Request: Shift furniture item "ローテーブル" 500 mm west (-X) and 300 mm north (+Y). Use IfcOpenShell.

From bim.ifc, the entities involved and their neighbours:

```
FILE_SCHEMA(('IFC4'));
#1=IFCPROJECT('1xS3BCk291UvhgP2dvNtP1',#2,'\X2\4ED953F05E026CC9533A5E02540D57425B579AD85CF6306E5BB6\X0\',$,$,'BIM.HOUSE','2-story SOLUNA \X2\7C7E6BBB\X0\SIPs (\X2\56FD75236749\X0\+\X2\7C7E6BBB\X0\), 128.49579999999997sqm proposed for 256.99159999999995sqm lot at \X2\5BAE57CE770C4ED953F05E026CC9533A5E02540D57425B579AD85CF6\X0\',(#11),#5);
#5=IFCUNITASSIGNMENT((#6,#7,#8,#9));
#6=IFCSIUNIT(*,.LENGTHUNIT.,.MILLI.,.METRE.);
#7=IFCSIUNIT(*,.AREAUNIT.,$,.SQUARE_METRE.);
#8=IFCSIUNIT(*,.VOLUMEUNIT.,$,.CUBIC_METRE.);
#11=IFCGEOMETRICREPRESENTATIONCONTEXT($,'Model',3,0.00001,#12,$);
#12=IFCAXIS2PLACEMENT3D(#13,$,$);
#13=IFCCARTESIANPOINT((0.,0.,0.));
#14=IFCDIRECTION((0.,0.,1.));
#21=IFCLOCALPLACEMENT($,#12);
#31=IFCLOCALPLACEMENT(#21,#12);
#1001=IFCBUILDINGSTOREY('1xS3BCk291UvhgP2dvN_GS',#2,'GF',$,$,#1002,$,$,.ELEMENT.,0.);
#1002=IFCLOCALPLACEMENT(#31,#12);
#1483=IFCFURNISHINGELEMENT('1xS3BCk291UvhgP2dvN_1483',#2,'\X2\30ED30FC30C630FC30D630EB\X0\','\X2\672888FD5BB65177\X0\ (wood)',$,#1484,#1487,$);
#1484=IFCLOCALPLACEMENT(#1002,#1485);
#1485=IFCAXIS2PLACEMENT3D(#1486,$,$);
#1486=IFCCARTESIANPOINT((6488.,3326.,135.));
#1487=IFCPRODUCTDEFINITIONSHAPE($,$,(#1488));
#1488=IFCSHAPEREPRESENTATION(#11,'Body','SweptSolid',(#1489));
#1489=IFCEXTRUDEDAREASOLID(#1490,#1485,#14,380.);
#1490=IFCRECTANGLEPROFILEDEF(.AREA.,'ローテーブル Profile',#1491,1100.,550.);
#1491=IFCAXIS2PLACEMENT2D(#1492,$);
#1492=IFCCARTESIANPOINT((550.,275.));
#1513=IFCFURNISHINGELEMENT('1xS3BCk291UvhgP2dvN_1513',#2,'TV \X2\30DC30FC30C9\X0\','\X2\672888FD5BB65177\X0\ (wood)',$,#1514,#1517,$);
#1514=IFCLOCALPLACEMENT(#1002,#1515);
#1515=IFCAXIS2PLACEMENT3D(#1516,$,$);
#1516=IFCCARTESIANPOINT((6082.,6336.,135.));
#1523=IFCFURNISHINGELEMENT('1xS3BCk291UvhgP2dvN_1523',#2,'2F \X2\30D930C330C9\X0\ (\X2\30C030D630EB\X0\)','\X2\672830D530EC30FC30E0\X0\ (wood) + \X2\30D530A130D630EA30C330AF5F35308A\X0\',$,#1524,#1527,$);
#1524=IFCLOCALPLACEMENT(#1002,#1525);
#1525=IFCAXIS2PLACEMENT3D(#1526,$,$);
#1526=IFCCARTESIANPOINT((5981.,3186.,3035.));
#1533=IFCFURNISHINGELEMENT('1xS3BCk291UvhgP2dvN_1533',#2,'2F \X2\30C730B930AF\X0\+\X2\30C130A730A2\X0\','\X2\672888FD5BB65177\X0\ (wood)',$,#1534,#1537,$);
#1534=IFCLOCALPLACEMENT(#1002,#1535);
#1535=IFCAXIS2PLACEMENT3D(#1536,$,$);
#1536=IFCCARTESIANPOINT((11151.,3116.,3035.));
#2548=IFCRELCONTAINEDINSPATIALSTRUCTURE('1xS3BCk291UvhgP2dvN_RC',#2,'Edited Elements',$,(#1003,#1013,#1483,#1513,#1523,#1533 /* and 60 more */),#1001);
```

```python
import ifcopenshell
import ifcopenshell.api.geometry
import ifcopenshell.util.placement
import ifcopenshell.util.unit

model = ifcopenshell.open("bim.ifc")
unit_scale = ifcopenshell.util.unit.calculate_unit_scale(model)

item = model.by_guid("1xS3BCk291UvhgP2dvN_1483")
matrix = ifcopenshell.util.placement.get_local_placement(item.ObjectPlacement)
matrix[0, 3] -= 0.5 / unit_scale
matrix[1, 3] += 0.3 / unit_scale
ifcopenshell.api.geometry.edit_object_placement(model, product=item, matrix=matrix, is_si=False)

print(ifcopenshell.util.placement.get_local_placement(item.ObjectPlacement).round(3) + 0.0)

model.write("bim_updated.ifc")
```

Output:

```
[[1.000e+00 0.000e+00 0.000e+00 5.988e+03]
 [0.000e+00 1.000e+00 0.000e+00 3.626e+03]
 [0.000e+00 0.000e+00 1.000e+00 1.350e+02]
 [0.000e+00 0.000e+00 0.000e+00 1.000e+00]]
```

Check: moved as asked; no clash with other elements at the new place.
